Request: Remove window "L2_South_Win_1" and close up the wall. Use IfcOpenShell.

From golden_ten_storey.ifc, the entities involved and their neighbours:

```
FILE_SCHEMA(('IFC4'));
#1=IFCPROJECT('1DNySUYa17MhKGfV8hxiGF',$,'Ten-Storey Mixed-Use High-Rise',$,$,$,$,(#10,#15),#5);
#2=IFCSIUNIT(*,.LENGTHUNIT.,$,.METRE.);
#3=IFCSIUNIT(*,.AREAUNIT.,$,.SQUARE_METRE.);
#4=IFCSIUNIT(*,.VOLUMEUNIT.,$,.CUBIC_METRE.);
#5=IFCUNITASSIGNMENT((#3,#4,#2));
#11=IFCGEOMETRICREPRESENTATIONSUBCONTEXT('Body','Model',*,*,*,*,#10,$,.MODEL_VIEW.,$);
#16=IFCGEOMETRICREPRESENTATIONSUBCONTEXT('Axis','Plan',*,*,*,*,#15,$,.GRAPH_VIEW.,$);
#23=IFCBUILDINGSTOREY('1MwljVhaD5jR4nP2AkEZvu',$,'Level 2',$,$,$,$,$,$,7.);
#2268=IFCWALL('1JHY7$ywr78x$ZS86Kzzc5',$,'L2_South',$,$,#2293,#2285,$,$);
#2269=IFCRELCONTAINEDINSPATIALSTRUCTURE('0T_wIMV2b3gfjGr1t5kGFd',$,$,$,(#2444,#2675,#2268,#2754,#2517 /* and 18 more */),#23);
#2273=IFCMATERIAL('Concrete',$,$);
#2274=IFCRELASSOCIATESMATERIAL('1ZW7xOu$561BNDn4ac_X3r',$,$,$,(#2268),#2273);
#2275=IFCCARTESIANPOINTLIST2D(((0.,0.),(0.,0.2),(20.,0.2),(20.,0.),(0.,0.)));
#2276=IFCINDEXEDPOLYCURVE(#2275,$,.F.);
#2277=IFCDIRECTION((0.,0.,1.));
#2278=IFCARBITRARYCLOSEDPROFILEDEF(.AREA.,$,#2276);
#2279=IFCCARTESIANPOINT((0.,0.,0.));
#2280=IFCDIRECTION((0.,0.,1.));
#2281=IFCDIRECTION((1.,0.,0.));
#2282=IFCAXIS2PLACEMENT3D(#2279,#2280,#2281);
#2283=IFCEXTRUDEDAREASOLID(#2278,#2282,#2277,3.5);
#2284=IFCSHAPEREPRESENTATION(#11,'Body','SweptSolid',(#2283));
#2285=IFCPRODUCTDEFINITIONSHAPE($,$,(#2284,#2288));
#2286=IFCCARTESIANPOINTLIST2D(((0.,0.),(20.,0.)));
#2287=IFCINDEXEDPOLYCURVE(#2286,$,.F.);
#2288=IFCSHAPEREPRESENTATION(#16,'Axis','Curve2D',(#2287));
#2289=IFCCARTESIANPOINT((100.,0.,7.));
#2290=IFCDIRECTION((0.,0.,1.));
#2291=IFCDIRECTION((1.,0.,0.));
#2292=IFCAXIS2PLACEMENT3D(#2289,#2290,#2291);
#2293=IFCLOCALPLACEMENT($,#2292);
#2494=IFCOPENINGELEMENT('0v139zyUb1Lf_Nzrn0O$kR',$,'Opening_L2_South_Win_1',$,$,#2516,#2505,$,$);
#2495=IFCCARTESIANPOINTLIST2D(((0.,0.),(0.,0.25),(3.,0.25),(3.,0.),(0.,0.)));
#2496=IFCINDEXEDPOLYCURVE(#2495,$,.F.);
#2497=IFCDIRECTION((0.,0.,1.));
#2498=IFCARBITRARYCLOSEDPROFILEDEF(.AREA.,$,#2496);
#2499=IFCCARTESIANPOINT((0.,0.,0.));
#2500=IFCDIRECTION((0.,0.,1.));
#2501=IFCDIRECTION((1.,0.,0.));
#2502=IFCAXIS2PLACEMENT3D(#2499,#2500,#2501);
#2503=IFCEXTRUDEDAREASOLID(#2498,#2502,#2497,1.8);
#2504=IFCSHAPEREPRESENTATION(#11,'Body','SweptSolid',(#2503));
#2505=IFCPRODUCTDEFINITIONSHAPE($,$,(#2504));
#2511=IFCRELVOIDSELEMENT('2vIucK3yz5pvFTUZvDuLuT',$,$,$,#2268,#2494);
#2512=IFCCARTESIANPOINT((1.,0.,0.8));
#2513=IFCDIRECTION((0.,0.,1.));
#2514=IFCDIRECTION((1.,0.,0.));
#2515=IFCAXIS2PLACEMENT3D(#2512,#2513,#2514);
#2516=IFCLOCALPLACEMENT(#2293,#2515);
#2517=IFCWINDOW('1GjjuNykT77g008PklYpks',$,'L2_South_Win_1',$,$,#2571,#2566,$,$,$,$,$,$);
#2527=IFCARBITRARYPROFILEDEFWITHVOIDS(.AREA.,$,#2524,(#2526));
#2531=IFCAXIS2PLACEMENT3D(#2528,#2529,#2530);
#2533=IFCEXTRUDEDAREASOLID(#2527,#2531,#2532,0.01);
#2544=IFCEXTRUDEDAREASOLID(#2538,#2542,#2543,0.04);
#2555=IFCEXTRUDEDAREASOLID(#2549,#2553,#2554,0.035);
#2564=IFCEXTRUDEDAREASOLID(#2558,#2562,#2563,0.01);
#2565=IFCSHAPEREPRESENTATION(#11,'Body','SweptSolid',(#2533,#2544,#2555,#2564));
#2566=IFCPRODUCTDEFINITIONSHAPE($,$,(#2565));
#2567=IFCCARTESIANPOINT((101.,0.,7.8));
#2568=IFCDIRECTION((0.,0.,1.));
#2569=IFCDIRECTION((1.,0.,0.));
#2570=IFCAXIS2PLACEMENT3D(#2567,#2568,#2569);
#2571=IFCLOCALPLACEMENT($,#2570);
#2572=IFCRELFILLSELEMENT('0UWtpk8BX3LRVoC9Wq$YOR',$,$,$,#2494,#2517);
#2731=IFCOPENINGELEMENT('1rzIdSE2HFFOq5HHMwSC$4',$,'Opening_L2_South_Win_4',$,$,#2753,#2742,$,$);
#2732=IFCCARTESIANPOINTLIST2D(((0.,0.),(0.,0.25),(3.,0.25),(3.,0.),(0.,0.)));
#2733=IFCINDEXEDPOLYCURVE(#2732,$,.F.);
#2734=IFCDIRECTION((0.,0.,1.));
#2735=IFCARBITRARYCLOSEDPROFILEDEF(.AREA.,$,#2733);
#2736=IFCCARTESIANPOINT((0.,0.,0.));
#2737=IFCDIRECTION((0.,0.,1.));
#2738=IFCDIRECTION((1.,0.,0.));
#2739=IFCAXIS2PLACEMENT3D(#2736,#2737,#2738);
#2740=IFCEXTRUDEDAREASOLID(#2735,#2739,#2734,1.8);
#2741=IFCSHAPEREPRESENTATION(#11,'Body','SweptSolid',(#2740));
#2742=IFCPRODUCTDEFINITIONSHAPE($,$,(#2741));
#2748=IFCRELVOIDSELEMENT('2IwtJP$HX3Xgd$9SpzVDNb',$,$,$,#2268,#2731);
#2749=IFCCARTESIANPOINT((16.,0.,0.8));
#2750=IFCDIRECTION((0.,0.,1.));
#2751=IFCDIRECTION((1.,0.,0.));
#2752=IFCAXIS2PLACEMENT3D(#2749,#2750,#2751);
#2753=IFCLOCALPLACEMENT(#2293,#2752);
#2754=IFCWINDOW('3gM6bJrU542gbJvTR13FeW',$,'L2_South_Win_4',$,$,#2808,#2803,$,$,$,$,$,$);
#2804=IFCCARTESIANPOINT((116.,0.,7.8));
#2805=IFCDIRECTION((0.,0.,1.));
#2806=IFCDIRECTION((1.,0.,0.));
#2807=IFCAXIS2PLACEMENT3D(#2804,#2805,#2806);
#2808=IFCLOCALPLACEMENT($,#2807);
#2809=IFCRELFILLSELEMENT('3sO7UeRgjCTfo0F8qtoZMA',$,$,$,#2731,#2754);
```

```python
import ifcopenshell
import ifcopenshell.api.feature
import ifcopenshell.api.root
import ifcopenshell.geom
import ifcopenshell.util.shape

model = ifcopenshell.open("golden_ten_storey.ifc")
settings = ifcopenshell.geom.settings()


def volume(element):
    """Net volume in cubic metres, openings subtracted."""
    shape = ifcopenshell.geom.create_shape(settings, element)
    return ifcopenshell.util.shape.get_volume(shape.geometry)


window = model.by_guid("1GjjuNykT77g008PklYpks")
opening = window.FillsVoids[0].RelatingOpeningElement
wall = opening.VoidsElements[0].RelatingBuildingElement
before = volume(wall)

ifcopenshell.api.root.remove_product(model, product=window)
ifcopenshell.api.feature.remove_feature(model, feature=opening)

after = volume(wall)

print(f"wall volume {before:.3f} -> {after:.3f} m3")

model.write("golden_ten_storey_rev.ifc")
```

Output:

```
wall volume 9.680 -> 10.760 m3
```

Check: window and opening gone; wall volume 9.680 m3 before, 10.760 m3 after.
